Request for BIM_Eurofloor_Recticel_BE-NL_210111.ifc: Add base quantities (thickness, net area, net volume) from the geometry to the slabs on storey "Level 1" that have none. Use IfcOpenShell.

First a look at what the model holds.

```python
import ifcopenshell
import ifcopenshell.util.element
import ifcopenshell.util.unit

model = ifcopenshell.open("BIM_Eurofloor_Recticel_BE-NL_210111.ifc")
print(model.schema)
for unit_type in ("LENGTHUNIT", "AREAUNIT", "VOLUMEUNIT"):
    print(unit_type, ifcopenshell.util.unit.calculate_unit_scale(model, unit_type))
storey = next(s for s in model.by_type("IfcBuildingStorey") if s.Name == "Level 1")
slabs = [e for e in ifcopenshell.util.element.get_decomposition(storey) if e.is_a("IfcSlab")]
for e in sorted(slabs, key=lambda e: e.id()):
    print(e.id(), e.is_a(), e.Name, list(ifcopenshell.util.element.get_psets(e, qtos_only=True)), sep=" | ")
```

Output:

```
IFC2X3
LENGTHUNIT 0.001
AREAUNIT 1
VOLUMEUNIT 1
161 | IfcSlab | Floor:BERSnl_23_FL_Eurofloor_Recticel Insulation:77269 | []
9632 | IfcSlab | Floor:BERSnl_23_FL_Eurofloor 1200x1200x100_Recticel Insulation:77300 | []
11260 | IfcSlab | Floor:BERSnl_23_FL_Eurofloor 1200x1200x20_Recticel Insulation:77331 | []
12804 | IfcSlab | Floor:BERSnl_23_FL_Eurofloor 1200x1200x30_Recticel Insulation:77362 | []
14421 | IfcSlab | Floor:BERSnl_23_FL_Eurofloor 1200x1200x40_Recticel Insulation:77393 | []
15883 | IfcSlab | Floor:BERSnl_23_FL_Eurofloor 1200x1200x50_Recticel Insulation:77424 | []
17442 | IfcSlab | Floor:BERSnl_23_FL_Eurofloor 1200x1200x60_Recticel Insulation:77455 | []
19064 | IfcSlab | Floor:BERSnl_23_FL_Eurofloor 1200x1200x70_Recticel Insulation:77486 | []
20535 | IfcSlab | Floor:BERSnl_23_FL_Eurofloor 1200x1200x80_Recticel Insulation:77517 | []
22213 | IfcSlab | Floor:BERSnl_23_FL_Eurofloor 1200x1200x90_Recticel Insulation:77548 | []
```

```python
import ifcopenshell
import ifcopenshell.api.pset
import ifcopenshell.geom
import ifcopenshell.util.element
import ifcopenshell.util.shape
import ifcopenshell.util.unit

model = ifcopenshell.open("BIM_Eurofloor_Recticel_BE-NL_210111.ifc")
unit_scale = ifcopenshell.util.unit.calculate_unit_scale(model)
area_scale = ifcopenshell.util.unit.calculate_unit_scale(model, "AREAUNIT")
volume_scale = ifcopenshell.util.unit.calculate_unit_scale(model, "VOLUMEUNIT")
settings = ifcopenshell.geom.settings()

storey = next(s for s in model.by_type("IfcBuildingStorey") if s.Name == "Level 1")
slabs = [e for e in ifcopenshell.util.element.get_decomposition(storey) if e.is_a("IfcSlab")]

for e in sorted(slabs, key=lambda e: e.id()):
    if ifcopenshell.util.element.get_psets(e, qtos_only=True, should_inherit=False):
        continue
    # Geometry comes back in metres, in the element's own axes.
    shape = ifcopenshell.geom.create_shape(settings, e)
    values = {
        "Width": ifcopenshell.util.shape.get_z(shape.geometry) / unit_scale,
        "NetArea": ifcopenshell.util.shape.get_footprint_area(shape.geometry) / area_scale,
        "NetVolume": ifcopenshell.util.shape.get_volume(shape.geometry) / volume_scale,
    }
    qto = ifcopenshell.api.pset.add_qto(model, product=e, name="BaseQuantities")
    ifcopenshell.api.pset.edit_qto(model, qto=qto, properties=values)
    print(e.id(), {k: round(v, 3) for k, v in values.items()})

model.write("BIM_Eurofloor_Recticel_BE-NL_210111_updated.ifc")
```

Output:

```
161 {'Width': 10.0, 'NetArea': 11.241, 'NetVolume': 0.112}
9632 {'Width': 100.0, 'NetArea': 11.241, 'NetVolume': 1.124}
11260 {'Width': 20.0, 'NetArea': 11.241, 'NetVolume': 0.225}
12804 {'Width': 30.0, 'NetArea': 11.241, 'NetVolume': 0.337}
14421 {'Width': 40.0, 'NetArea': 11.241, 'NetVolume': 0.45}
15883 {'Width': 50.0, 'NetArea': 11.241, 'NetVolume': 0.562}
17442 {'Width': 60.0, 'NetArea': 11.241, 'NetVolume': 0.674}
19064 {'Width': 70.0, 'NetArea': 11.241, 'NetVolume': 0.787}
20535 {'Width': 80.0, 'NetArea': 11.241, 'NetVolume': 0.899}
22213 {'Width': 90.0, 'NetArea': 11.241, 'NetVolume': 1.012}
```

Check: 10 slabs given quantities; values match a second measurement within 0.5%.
